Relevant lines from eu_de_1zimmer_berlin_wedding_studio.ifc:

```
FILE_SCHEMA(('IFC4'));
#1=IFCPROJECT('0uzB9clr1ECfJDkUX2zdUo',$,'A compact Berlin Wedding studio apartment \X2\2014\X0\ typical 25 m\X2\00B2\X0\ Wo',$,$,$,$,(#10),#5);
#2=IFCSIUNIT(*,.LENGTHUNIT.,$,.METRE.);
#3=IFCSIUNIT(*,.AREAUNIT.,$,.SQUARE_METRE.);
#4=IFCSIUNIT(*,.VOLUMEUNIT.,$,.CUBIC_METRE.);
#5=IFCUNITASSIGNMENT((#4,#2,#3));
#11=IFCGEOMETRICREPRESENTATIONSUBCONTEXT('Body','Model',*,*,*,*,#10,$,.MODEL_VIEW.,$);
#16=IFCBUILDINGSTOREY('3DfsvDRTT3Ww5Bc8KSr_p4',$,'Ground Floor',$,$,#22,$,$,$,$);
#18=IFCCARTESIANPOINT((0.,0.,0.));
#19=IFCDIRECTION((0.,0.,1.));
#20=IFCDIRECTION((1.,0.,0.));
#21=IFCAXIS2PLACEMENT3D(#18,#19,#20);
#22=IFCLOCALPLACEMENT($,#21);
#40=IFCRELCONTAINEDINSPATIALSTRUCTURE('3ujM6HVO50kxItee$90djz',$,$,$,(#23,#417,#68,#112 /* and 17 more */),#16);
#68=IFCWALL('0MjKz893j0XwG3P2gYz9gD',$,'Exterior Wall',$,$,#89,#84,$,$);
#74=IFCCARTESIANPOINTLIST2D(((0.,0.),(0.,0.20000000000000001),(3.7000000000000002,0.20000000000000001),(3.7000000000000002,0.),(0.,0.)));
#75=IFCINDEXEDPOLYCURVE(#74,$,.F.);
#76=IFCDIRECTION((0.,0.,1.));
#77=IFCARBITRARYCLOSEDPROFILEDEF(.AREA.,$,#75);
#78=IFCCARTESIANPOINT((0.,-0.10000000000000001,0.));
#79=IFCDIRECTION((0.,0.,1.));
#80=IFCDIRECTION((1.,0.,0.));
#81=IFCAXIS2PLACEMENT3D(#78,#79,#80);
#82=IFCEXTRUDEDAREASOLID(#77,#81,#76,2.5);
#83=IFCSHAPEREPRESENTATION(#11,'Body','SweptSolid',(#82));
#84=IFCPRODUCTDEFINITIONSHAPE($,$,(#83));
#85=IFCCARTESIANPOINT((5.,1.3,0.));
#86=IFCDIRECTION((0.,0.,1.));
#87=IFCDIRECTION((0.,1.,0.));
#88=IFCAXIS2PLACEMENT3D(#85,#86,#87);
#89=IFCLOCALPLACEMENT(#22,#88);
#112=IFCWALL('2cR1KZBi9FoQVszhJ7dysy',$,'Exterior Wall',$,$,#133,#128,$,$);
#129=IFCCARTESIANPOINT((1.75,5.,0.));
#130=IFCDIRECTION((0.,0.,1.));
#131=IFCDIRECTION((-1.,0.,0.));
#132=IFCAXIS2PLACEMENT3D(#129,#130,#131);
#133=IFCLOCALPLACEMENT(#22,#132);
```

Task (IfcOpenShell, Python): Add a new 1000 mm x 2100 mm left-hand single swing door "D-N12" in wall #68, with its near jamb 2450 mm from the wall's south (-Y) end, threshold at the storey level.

```python
import numpy as np
import ifcopenshell
import ifcopenshell.api.feature
import ifcopenshell.api.geometry
import ifcopenshell.api.root
import ifcopenshell.api.spatial
import ifcopenshell.geom
import ifcopenshell.util.element
import ifcopenshell.util.placement
import ifcopenshell.util.representation
import ifcopenshell.util.shape
import ifcopenshell.util.unit

model = ifcopenshell.open("eu_de_1zimmer_berlin_wedding_studio.ifc")
unit_scale = ifcopenshell.util.unit.calculate_unit_scale(model)
settings = ifcopenshell.geom.settings()


def volume(element):
    """Net volume in cubic metres, openings subtracted."""
    shape = ifcopenshell.geom.create_shape(settings, element)
    return ifcopenshell.util.shape.get_volume(shape.geometry)


wall = model.by_guid("0MjKz893j0XwG3P2gYz9gD")
storey = ifcopenshell.util.element.get_container(wall, ifc_class="IfcBuildingStorey")
context = ifcopenshell.util.representation.get_context(model, "Model", "Body", "MODEL_VIEW")
before = volume(wall)

width, height, from_end, sill = 1, 2.1, 2.45, 0.0  # metres

# The wall runs along its own X axis, and the end named is its -X end.
wall_shape = ifcopenshell.geom.create_shape(settings, wall)
x, y, z = ifcopenshell.util.shape.get_vertices(wall_shape.geometry).T
start = x.min() + from_end
face, thickness = float(y.min()), float(y.max() - y.min())
wall_matrix = ifcopenshell.util.placement.get_local_placement(wall.ObjectPlacement)
level = ifcopenshell.util.placement.get_local_placement(storey.ObjectPlacement)[2, 3]


def in_wall(x, y):
    """Placement at x, y metres in the wall's axes, at sill height."""
    matrix = wall_matrix.copy()
    matrix[:, 3] = wall_matrix @ np.array([x / unit_scale, y / unit_scale, 0.0, 1.0])
    matrix[2, 3] = level + sill / unit_scale
    return matrix


# Opening: a box that overshoots both wall faces by 50 mm.
opening = ifcopenshell.api.root.create_entity(model, ifc_class="IfcOpeningElement", predefined_type="OPENING")
box = ifcopenshell.api.geometry.add_wall_representation(
    model, context=context, length=width, height=height, thickness=thickness + 0.1
)
ifcopenshell.api.geometry.assign_representation(model, product=opening, representation=box)
ifcopenshell.api.geometry.edit_object_placement(model, product=opening, matrix=in_wall(start, face - 0.05), is_si=False)
ifcopenshell.api.feature.add_feature(model, feature=opening, element=wall)

door = ifcopenshell.api.root.create_entity(model, ifc_class="IfcDoor", name="D-N12", predefined_type="DOOR")
door.OverallWidth, door.OverallHeight = width / unit_scale, height / unit_scale
door.OperationType = "SINGLE_SWING_LEFT"
body = ifcopenshell.api.geometry.add_door_representation(
    model,
    context=context,
    overall_width=door.OverallWidth,
    overall_height=door.OverallHeight,
    operation_type="SINGLE_SWING_LEFT",
    lining_properties={"LiningDepth": thickness / unit_scale, "ThresholdDepth": thickness / unit_scale},
)
ifcopenshell.api.geometry.assign_representation(model, product=door, representation=body)
ifcopenshell.api.spatial.assign_container(model, products=[door], relating_structure=storey)
ifcopenshell.api.feature.add_filling(model, opening=opening, element=door)

# The lining spans the wall, so the door starts at the wall face.
ifcopenshell.api.geometry.edit_object_placement(model, product=door, matrix=in_wall(start, face), is_si=False)

after = volume(wall)

print(f"wall volume {before:.3f} -> {after:.3f} m3")

model.write("eu_de_1zimmer_berlin_wedding_studio_v2.ifc")
```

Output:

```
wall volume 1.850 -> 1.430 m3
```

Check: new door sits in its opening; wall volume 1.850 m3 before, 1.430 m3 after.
